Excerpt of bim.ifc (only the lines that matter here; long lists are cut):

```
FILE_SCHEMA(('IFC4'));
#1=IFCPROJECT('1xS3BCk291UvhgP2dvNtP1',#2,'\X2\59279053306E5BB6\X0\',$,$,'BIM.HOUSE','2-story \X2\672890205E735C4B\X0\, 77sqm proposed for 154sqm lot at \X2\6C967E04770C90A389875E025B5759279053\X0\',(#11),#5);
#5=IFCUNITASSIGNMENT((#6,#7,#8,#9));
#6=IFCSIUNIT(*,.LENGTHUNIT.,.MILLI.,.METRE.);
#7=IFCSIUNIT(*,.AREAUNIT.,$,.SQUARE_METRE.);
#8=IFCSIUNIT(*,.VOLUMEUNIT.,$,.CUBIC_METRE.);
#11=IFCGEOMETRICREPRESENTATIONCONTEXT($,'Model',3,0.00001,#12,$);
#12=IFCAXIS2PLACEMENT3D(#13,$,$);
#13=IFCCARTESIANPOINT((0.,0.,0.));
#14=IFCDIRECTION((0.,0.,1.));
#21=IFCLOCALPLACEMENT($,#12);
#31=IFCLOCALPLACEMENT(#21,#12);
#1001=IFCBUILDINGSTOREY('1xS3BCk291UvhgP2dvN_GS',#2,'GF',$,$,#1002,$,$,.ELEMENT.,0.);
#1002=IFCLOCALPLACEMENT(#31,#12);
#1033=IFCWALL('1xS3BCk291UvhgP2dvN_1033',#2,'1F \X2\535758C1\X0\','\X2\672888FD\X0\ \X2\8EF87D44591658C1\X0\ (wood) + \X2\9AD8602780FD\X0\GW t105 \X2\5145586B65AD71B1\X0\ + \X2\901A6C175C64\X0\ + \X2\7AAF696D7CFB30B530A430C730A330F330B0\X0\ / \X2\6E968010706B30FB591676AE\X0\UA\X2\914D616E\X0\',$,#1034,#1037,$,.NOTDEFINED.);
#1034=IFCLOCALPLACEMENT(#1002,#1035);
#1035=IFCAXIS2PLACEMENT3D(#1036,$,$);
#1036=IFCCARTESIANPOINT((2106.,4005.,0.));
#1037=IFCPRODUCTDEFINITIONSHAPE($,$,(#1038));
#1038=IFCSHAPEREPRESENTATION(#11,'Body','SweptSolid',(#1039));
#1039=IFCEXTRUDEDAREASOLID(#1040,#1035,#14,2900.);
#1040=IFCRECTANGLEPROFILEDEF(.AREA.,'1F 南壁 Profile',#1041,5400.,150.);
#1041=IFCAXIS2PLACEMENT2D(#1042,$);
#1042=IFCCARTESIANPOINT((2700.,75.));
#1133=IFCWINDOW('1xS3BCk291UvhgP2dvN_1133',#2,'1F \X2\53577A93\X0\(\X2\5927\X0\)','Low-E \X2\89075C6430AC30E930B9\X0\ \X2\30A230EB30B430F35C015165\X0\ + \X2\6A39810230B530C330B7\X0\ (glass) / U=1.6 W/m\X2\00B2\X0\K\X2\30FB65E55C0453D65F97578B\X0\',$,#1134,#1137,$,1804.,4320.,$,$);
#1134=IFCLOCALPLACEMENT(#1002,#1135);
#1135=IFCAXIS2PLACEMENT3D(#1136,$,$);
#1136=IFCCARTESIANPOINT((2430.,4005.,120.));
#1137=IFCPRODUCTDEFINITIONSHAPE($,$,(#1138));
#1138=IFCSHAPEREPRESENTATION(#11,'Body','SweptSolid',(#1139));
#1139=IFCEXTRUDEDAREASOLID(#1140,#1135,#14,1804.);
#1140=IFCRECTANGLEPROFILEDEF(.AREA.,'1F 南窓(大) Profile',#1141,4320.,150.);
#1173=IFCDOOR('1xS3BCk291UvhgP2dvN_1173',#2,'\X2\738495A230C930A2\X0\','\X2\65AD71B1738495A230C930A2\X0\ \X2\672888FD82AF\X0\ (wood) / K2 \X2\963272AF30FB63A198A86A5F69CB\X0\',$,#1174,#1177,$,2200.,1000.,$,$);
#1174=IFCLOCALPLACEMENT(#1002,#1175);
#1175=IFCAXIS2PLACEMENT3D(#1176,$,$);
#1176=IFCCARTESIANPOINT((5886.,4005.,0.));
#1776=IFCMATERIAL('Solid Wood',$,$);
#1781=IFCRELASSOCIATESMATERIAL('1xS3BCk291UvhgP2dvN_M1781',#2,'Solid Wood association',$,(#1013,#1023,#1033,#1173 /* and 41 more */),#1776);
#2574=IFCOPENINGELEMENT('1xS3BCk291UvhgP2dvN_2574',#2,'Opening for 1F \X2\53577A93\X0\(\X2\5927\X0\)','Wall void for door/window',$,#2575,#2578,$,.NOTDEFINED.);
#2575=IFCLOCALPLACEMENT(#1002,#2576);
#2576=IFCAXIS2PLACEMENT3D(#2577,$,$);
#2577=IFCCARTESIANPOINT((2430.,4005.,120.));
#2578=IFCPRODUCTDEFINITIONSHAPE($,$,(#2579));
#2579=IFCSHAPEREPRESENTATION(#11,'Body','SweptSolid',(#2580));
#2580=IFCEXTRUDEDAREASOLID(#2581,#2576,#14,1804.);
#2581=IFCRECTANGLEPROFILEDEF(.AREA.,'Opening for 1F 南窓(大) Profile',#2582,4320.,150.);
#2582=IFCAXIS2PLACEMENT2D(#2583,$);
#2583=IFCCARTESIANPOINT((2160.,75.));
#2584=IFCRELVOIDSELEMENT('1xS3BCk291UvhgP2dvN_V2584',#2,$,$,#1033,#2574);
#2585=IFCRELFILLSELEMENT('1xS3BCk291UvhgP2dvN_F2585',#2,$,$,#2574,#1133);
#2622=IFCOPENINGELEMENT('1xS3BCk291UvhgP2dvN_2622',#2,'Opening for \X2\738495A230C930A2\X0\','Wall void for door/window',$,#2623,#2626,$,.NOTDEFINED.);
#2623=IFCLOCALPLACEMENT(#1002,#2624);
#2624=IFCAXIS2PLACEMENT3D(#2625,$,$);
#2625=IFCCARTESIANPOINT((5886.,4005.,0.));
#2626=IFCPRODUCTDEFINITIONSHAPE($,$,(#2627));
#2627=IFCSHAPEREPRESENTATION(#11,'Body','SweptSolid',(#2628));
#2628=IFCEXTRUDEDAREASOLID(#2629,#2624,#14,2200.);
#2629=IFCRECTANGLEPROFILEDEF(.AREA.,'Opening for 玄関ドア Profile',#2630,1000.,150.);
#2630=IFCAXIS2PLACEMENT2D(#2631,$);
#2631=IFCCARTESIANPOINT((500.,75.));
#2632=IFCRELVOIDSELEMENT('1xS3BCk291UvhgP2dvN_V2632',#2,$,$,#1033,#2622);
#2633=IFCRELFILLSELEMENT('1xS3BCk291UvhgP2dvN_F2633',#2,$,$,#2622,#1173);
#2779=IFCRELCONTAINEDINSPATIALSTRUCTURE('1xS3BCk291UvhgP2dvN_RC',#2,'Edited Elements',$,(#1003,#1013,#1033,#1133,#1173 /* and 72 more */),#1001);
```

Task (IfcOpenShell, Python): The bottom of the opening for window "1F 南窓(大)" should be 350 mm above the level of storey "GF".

```python
import numpy as np
import ifcopenshell
import ifcopenshell.api.geometry
import ifcopenshell.geom
import ifcopenshell.util.element
import ifcopenshell.util.placement
import ifcopenshell.util.shape
import ifcopenshell.util.unit

model = ifcopenshell.open("bim.ifc")
unit_scale = ifcopenshell.util.unit.calculate_unit_scale(model)

window = model.by_guid("1xS3BCk291UvhgP2dvN_1133")
opening = window.FillsVoids[0].RelatingOpeningElement
storey = ifcopenshell.util.element.get_container(window, ifc_class="IfcBuildingStorey")
level = ifcopenshell.util.placement.get_local_placement(storey.ObjectPlacement)[2, 3]

# The opening's origin need not be at the sill, so measure its lowest point.
shape = ifcopenshell.geom.create_shape(ifcopenshell.geom.settings(), opening)
bottom = ifcopenshell.util.shape.get_shape_bottom_elevation(shape, shape.geometry) / unit_scale
dz = level + 0.35 / unit_scale - bottom

shift = np.array([0.0, 0.0, dz])
# The window is not placed relative to its opening, so move both.
for product in (opening, window):
    matrix = ifcopenshell.util.placement.get_local_placement(product.ObjectPlacement)
    matrix[:3, 3] += shift
    ifcopenshell.api.geometry.edit_object_placement(model, product=product, matrix=matrix, is_si=False)

print(f"moved by {dz * unit_scale:+.3f} m")

model.write("bim_rev.ifc")
```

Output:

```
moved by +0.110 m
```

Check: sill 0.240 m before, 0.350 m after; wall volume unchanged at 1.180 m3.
